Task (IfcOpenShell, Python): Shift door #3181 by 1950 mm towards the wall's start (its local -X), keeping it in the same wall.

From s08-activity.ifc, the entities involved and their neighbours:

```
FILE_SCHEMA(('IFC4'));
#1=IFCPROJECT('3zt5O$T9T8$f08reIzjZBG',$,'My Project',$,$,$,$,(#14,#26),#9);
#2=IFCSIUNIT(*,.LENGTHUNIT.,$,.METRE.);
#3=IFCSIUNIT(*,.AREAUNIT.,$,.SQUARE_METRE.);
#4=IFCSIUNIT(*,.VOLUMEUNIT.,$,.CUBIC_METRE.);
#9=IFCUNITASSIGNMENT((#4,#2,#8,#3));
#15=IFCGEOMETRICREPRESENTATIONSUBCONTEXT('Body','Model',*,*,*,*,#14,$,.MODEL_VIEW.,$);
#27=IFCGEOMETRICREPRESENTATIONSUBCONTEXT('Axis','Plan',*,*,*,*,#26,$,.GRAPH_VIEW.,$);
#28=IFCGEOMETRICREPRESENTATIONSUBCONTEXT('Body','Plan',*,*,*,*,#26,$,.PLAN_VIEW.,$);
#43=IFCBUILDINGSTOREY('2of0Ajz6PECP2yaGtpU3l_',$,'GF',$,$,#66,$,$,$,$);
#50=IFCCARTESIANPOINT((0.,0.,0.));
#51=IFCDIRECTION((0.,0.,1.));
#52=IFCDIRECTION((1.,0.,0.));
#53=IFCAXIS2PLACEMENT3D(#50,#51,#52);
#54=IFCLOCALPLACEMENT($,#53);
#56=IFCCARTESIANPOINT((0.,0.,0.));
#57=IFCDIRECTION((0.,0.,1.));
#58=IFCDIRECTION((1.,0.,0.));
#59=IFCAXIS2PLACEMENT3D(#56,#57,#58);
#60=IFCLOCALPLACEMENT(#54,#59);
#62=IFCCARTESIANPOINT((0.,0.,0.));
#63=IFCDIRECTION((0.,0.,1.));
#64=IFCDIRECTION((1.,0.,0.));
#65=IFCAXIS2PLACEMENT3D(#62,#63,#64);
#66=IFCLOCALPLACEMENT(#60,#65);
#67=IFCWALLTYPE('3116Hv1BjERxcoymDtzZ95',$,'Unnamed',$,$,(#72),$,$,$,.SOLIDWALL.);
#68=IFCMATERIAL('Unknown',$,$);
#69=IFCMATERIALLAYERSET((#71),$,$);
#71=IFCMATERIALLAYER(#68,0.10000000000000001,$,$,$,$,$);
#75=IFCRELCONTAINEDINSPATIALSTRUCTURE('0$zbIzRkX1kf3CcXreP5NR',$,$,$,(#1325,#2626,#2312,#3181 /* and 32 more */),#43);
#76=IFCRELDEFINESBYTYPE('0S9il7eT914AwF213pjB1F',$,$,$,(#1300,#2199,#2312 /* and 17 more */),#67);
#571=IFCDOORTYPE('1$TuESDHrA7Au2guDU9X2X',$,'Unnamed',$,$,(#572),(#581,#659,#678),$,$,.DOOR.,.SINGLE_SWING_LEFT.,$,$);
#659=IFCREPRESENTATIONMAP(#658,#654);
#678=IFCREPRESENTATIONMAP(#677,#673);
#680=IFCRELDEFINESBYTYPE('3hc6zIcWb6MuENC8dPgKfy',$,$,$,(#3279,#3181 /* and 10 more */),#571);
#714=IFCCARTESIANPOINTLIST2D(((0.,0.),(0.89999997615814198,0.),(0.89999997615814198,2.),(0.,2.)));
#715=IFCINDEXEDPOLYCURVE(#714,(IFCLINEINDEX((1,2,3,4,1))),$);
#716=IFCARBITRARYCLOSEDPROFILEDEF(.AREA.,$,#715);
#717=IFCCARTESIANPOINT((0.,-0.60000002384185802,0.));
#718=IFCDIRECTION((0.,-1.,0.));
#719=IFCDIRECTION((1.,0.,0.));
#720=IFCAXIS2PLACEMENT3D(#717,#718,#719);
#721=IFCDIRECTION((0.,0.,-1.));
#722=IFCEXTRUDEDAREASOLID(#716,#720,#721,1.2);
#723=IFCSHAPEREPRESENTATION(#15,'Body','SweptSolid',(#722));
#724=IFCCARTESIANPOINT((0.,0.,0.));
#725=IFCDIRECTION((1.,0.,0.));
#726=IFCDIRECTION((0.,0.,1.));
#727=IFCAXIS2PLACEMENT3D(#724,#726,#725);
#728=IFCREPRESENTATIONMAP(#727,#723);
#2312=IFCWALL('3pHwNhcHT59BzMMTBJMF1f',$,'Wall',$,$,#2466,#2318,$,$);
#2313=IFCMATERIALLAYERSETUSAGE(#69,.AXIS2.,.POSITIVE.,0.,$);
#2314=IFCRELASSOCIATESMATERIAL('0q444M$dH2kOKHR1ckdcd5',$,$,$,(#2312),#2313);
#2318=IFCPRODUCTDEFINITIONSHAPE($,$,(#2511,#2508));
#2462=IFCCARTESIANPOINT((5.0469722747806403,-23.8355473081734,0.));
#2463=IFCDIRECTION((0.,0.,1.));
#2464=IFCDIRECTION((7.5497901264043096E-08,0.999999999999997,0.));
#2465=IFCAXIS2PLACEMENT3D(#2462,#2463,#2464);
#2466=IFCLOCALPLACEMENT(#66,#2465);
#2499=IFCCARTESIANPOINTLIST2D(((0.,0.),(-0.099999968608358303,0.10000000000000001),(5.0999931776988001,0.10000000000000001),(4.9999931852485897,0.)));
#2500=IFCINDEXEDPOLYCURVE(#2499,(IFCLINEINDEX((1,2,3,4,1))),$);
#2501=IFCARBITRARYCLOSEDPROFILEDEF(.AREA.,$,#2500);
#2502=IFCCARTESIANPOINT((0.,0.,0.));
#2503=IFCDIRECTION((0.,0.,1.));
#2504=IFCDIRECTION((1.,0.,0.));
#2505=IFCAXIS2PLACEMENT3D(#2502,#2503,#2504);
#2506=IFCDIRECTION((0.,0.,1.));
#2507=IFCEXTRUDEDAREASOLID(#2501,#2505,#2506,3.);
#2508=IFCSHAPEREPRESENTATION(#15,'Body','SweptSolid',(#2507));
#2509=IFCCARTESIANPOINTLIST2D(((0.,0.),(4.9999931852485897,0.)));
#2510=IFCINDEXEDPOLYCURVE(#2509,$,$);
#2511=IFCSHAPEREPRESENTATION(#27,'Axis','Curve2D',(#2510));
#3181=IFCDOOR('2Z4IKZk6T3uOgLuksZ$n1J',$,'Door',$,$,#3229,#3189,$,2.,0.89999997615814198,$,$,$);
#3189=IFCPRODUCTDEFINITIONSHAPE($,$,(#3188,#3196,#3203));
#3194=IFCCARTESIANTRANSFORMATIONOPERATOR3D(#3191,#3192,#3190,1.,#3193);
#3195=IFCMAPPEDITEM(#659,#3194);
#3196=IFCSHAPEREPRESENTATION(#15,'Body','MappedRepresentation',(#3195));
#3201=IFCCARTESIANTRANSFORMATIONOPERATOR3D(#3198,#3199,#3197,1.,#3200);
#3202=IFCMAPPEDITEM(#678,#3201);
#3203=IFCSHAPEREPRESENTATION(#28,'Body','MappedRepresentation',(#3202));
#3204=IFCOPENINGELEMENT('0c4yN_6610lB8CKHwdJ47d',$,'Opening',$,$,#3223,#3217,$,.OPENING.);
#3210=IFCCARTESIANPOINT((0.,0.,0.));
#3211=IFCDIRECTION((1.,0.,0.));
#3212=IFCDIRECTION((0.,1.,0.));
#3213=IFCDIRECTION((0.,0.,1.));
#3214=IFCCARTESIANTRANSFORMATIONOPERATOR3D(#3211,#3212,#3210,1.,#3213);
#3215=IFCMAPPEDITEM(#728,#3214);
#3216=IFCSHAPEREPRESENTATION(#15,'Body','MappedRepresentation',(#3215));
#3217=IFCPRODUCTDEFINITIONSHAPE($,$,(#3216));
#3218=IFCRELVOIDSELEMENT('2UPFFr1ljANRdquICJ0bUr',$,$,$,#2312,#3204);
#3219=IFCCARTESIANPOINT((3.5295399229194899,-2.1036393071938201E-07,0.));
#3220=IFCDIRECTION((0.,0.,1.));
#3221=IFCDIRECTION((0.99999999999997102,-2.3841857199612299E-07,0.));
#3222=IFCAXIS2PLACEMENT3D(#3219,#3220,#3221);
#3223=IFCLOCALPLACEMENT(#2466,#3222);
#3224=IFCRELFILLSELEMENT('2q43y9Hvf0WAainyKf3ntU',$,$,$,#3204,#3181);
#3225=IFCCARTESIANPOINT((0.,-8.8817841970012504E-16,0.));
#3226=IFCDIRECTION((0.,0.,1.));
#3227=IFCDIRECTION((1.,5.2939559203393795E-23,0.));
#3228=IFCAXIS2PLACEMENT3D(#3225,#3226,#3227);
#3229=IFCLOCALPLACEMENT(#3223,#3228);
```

```python
import ifcopenshell
import ifcopenshell.api.geometry
import ifcopenshell.util.placement
import ifcopenshell.util.unit

model = ifcopenshell.open("s08-activity.ifc")
unit_scale = ifcopenshell.util.unit.calculate_unit_scale(model)

door = model.by_guid("2Z4IKZk6T3uOgLuksZ$n1J")
opening = door.FillsVoids[0].RelatingOpeningElement
wall = opening.VoidsElements[0].RelatingBuildingElement

wall_matrix = ifcopenshell.util.placement.get_local_placement(wall.ObjectPlacement)
shift = wall_matrix[:3, 0] * -1.95 / unit_scale
before = ifcopenshell.util.placement.get_local_placement(door.ObjectPlacement)[:3, 3].copy()

# The door is placed relative to its opening, so it follows when the opening moves.
matrix = ifcopenshell.util.placement.get_local_placement(opening.ObjectPlacement)
matrix[:3, 3] += shift
ifcopenshell.api.geometry.edit_object_placement(
    model, product=opening, matrix=matrix, is_si=False, should_transform_children=True
)

after = ifcopenshell.util.placement.get_local_placement(door.ObjectPlacement)[:3, 3]
print("door moved by", (after - before).round(3) + 0.0)

model.write("s08-activity_edited.ifc")
```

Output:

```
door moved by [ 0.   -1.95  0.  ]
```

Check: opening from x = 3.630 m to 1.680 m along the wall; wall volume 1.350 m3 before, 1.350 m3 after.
